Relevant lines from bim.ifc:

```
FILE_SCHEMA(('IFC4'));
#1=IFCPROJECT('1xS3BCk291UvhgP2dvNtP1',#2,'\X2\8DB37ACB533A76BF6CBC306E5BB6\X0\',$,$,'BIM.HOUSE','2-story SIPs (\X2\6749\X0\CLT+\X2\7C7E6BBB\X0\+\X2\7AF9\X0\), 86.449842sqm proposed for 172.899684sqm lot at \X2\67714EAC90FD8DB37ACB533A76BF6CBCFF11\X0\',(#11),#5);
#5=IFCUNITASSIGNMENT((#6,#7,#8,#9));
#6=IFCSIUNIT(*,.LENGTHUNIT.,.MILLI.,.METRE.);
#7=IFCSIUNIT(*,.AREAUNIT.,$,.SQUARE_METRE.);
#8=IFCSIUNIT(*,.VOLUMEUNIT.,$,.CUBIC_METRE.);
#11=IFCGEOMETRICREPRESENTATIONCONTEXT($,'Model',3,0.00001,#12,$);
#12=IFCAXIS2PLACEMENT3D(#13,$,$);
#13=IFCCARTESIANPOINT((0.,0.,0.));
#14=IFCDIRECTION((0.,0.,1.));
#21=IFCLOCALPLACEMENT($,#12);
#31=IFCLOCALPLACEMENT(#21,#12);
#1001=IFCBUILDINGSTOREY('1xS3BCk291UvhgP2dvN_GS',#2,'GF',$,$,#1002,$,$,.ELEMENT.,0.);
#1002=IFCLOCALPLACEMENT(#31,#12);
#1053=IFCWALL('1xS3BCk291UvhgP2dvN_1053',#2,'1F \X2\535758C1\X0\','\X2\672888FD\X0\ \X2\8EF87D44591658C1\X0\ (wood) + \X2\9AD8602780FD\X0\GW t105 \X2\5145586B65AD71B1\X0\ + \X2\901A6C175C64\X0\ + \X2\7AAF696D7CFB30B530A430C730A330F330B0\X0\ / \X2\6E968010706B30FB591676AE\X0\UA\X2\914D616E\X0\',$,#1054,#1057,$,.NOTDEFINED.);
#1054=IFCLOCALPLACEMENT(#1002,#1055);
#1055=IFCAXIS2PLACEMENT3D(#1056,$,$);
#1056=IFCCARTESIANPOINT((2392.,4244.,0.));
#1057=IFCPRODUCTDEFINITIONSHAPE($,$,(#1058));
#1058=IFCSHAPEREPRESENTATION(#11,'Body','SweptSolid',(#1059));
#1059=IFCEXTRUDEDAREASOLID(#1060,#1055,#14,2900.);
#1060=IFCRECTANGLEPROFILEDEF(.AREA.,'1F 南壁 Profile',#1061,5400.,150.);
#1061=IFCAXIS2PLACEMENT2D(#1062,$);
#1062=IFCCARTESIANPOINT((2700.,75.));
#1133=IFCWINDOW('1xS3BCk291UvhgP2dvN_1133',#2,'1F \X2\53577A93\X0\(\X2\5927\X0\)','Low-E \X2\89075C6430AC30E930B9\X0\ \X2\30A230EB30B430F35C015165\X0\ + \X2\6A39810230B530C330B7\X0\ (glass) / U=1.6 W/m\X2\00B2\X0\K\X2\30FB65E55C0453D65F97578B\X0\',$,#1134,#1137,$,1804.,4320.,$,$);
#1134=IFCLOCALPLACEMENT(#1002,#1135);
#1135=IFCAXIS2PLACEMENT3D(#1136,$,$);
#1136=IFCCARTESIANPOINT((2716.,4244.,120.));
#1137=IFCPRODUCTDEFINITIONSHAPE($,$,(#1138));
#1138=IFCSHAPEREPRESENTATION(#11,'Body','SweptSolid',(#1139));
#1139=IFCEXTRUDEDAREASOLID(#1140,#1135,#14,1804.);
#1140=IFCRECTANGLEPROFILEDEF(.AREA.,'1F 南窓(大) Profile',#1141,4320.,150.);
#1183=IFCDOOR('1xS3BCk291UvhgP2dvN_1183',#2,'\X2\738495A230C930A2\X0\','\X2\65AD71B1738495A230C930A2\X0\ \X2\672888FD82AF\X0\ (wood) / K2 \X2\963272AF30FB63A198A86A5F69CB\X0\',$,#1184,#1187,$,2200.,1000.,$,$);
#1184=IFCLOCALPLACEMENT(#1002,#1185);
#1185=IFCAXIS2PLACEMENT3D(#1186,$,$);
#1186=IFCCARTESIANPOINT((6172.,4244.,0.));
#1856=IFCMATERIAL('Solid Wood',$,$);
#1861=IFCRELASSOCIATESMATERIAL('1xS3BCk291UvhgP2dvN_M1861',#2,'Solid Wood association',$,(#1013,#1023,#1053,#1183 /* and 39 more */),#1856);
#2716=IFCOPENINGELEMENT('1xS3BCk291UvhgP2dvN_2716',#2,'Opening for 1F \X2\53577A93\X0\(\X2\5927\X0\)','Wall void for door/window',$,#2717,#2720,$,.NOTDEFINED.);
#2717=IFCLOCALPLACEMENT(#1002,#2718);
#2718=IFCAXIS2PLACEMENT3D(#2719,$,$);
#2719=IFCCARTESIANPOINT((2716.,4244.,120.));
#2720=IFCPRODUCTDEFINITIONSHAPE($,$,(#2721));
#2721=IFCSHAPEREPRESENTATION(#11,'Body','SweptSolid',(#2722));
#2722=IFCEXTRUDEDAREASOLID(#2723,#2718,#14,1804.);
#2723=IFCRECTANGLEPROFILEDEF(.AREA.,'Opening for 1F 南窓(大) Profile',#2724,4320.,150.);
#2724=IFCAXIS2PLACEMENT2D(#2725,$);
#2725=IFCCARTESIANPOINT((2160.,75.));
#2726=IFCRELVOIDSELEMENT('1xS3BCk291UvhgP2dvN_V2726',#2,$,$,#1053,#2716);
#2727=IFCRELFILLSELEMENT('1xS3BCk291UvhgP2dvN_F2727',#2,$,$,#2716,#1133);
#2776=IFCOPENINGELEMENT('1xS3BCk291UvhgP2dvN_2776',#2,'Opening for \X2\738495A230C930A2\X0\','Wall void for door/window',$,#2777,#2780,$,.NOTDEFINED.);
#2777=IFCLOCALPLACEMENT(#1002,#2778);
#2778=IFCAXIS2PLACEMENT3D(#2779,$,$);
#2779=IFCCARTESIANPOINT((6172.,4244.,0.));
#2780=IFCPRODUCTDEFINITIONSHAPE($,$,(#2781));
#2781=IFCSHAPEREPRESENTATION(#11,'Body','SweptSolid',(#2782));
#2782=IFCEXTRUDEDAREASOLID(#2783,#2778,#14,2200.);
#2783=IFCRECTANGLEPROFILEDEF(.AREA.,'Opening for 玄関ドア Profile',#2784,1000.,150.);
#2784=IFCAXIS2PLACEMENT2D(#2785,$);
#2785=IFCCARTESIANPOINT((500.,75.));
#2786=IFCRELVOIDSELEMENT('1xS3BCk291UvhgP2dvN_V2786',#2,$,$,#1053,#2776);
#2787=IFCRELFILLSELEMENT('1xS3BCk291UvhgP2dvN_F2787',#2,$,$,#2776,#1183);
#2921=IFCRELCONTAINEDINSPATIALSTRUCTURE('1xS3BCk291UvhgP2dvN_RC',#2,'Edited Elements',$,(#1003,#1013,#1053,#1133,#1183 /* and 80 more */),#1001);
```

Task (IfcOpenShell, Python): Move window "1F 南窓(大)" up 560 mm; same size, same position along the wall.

```python
import numpy as np
import ifcopenshell
import ifcopenshell.api.geometry
import ifcopenshell.util.placement
import ifcopenshell.util.unit

model = ifcopenshell.open("bim.ifc")
unit_scale = ifcopenshell.util.unit.calculate_unit_scale(model)

window = model.by_guid("1xS3BCk291UvhgP2dvN_1133")
opening = window.FillsVoids[0].RelatingOpeningElement
dz = 0.56 / unit_scale

shift = np.array([0.0, 0.0, dz])
# The window is not placed relative to its opening, so move both.
for product in (opening, window):
    matrix = ifcopenshell.util.placement.get_local_placement(product.ObjectPlacement)
    matrix[:3, 3] += shift
    ifcopenshell.api.geometry.edit_object_placement(model, product=product, matrix=matrix, is_si=False)

print(f"moved by {dz * unit_scale:+.3f} m")

model.write("bim_v2.ifc")
```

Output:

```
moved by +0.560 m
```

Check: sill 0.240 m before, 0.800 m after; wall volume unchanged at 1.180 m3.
